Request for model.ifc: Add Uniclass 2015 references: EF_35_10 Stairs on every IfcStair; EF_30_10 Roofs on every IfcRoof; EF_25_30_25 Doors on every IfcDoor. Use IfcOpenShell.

First a look at what the model holds.

```python
import ifcopenshell

model = ifcopenshell.open("model.ifc")
print(model.schema)
print("classifications:", [c.Name for c in model.by_type("IfcClassification")])
for ifc_class in ("IfcDoor", "IfcRoof", "IfcStair", "IfcWall", "IfcWindow"):
    print(ifc_class, len(model.by_type(ifc_class)))
```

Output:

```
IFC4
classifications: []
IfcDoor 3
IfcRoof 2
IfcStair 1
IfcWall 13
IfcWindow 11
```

```python
import ifcopenshell
import ifcopenshell.api.classification

model = ifcopenshell.open("model.ifc")

system = ifcopenshell.api.classification.add_classification(model, classification="Uniclass 2015")

codes = {
    "IfcStair": ("EF_35_10", "Stairs"),
    "IfcRoof": ("EF_30_10", "Roofs"),
    "IfcDoor": ("EF_25_30_25", "Doors"),
}
for ifc_class, (code, name) in codes.items():
    products = model.by_type(ifc_class)
    ifcopenshell.api.classification.add_reference(
        model, products=products, classification=system, identification=code, name=name
    )
    print(code, len(products))

model.write("model-out.ifc")
```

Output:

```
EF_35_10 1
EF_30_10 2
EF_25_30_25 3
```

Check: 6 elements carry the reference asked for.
